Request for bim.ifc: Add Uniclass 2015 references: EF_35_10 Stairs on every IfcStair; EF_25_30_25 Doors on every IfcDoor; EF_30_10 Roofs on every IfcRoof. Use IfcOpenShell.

First a look at what the model holds.

```python
import ifcopenshell

model = ifcopenshell.open("bim.ifc")
print(model.schema)
print("classifications:", [c.Name for c in model.by_type("IfcClassification")])
for ifc_class in ("IfcDoor", "IfcRoof", "IfcStair", "IfcWall", "IfcWindow"):
    print(ifc_class, len(model.by_type(ifc_class)))
```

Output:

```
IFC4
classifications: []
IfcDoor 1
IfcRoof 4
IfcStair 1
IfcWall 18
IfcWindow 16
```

```python
import ifcopenshell
import ifcopenshell.api.classification

model = ifcopenshell.open("bim.ifc")

system = ifcopenshell.api.classification.add_classification(model, classification="Uniclass 2015")

codes = {
    "IfcStair": ("EF_35_10", "Stairs"),
    "IfcDoor": ("EF_25_30_25", "Doors"),
    "IfcRoof": ("EF_30_10", "Roofs"),
}
for ifc_class, (code, name) in codes.items():
    products = model.by_type(ifc_class)
    ifcopenshell.api.classification.add_reference(
        model, products=products, classification=system, identification=code, name=name
    )
    print(code, len(products))

model.write("bim-out.ifc")
```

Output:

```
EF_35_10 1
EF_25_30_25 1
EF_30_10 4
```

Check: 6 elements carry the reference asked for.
